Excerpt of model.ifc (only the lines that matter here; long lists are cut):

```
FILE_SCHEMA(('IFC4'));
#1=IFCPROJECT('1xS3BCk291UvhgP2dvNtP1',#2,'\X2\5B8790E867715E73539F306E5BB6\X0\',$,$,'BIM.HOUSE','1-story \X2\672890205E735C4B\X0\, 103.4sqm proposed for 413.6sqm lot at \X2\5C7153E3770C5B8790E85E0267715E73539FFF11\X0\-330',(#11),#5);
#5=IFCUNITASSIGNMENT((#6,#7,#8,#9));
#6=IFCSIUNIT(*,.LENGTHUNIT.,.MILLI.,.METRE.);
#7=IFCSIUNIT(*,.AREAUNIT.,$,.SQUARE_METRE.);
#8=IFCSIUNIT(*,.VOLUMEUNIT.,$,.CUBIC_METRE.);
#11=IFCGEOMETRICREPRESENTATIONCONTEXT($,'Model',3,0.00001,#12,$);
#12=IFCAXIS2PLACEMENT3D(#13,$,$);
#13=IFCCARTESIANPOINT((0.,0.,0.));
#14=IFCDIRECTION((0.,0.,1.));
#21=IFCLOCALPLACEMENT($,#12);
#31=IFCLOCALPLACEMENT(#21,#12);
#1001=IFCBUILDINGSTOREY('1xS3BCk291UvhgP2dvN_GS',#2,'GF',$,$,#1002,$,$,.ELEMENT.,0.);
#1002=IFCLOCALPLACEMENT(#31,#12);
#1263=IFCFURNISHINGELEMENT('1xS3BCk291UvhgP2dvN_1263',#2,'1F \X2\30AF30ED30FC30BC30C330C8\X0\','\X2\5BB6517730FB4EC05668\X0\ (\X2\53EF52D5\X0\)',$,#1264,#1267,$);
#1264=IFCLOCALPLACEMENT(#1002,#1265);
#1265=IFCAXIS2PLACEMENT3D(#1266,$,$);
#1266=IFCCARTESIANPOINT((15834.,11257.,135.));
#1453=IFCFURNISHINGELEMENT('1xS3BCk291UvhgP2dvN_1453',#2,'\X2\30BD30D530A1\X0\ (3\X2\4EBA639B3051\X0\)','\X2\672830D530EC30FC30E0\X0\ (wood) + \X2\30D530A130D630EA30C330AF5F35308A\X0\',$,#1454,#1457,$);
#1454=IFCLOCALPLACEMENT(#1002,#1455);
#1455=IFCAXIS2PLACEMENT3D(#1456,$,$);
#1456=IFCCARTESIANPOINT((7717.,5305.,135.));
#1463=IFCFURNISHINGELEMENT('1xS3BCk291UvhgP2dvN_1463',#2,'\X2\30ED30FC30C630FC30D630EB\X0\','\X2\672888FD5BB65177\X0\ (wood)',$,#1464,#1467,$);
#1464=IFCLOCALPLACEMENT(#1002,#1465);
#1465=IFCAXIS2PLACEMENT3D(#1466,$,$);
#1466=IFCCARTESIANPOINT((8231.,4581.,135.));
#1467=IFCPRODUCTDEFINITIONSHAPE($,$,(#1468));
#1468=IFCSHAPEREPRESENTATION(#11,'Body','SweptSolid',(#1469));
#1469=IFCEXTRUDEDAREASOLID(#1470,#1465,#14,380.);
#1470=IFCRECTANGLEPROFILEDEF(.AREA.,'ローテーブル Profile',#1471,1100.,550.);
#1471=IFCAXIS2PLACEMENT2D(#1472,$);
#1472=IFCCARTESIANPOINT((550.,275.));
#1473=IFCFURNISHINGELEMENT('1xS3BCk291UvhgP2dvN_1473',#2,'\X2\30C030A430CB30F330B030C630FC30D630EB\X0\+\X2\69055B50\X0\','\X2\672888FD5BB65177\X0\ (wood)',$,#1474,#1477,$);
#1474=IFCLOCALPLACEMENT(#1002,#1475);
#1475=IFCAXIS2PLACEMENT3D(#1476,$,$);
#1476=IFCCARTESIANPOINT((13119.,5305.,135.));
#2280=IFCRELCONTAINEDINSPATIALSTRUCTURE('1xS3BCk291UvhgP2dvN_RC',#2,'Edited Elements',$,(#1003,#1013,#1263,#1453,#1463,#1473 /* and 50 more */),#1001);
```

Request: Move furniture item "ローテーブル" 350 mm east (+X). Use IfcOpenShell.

```python
import ifcopenshell
import ifcopenshell.api.geometry
import ifcopenshell.util.placement

model = ifcopenshell.open("model.ifc")

item = model.by_guid("1xS3BCk291UvhgP2dvN_1463")
matrix = ifcopenshell.util.placement.get_local_placement(item.ObjectPlacement)
matrix[0, 3] += 350.0
ifcopenshell.api.geometry.edit_object_placement(model, product=item, matrix=matrix, is_si=False)

print(ifcopenshell.util.placement.get_local_placement(item.ObjectPlacement).round(3) + 0.0)

model.write("model_updated.ifc")
```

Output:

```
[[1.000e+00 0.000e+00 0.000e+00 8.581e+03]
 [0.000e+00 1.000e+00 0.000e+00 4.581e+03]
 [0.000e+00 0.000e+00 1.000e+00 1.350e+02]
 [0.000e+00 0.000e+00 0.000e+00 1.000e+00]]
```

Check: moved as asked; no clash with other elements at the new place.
